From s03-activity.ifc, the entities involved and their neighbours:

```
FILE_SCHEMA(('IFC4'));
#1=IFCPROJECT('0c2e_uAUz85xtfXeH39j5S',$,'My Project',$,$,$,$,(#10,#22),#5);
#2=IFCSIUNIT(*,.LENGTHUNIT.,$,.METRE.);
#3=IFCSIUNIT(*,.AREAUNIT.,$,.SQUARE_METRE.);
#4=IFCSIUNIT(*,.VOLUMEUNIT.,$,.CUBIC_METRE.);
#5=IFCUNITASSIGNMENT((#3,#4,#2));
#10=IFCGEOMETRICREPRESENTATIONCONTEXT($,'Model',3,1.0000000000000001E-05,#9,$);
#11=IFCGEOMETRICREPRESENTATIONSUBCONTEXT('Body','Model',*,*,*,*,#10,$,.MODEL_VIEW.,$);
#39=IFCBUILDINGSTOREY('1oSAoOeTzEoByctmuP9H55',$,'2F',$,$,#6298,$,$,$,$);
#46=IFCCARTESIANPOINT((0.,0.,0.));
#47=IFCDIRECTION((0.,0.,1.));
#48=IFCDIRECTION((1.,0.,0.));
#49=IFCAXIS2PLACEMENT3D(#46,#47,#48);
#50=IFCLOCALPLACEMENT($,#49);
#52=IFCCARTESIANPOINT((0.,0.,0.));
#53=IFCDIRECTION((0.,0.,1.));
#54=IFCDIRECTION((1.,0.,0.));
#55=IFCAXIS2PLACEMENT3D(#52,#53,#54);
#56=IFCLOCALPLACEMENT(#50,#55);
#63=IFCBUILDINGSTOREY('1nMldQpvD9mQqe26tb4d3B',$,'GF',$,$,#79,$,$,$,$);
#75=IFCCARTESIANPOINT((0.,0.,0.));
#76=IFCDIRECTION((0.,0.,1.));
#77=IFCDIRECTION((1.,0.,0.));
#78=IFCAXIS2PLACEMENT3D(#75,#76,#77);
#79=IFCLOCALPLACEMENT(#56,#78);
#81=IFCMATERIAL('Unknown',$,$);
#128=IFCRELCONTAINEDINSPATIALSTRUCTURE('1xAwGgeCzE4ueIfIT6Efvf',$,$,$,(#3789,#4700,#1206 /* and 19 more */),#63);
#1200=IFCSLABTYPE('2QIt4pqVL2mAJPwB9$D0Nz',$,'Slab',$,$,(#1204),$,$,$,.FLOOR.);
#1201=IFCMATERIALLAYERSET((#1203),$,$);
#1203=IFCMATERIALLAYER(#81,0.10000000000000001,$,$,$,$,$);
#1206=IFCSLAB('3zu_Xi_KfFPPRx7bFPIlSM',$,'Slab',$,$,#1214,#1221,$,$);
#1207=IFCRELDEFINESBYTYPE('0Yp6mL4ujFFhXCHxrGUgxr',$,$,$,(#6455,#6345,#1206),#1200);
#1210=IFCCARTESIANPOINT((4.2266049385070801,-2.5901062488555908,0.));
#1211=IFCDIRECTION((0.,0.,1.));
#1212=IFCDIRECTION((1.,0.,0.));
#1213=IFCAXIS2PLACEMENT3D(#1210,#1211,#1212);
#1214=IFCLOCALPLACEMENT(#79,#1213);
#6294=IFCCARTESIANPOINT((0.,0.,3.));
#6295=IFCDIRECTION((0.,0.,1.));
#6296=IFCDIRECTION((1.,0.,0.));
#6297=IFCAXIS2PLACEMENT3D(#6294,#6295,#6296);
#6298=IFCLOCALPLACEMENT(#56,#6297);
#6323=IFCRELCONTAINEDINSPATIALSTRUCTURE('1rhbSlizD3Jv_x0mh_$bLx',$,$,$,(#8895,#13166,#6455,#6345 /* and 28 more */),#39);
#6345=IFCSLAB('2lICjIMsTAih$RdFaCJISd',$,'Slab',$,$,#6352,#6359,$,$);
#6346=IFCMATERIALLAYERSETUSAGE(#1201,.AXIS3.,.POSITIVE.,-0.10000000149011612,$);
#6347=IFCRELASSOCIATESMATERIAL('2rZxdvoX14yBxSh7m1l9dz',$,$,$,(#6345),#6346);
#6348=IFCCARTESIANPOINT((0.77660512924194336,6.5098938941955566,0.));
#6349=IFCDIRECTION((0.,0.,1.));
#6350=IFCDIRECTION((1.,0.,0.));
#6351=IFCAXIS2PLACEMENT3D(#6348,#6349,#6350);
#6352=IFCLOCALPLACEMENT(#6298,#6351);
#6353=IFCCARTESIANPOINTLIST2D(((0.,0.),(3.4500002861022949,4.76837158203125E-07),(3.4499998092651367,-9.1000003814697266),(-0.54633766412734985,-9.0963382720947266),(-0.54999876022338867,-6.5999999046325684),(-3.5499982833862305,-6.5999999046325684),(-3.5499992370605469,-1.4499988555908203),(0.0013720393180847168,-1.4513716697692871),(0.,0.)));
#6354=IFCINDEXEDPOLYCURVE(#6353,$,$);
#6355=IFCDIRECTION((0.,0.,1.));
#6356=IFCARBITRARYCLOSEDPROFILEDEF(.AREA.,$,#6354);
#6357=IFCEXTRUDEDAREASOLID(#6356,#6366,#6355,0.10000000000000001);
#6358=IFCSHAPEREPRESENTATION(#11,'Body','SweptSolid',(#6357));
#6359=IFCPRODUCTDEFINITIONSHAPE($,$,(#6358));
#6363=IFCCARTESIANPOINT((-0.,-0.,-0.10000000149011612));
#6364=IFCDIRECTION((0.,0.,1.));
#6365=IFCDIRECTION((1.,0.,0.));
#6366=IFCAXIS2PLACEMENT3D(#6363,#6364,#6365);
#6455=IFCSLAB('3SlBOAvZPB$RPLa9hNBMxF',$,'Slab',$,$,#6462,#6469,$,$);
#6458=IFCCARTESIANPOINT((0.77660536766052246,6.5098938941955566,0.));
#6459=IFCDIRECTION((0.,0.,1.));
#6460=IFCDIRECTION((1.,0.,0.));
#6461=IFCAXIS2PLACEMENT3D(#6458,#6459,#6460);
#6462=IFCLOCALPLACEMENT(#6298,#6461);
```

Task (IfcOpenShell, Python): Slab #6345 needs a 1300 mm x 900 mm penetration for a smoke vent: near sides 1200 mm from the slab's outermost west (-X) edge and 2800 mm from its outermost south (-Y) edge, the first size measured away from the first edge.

```python
import numpy as np
import ifcopenshell
import ifcopenshell.api.feature
import ifcopenshell.api.geometry
import ifcopenshell.api.root
import ifcopenshell.geom
import ifcopenshell.util.placement
import ifcopenshell.util.representation
import ifcopenshell.util.shape
import ifcopenshell.util.unit

model = ifcopenshell.open("s03-activity.ifc")
unit_scale = ifcopenshell.util.unit.calculate_unit_scale(model)
settings = ifcopenshell.geom.settings()


def volume(element):
    """Net volume in cubic metres, openings subtracted."""
    shape = ifcopenshell.geom.create_shape(settings, element)
    return ifcopenshell.util.shape.get_volume(shape.geometry)


slab = model.by_guid("2lICjIMsTAih$RdFaCJISd")
before = volume(slab)

# Extent in the slab's own axes, in metres. The edges named are its -X and -Y sides.
slab_shape = ifcopenshell.geom.create_shape(settings, slab)
vertices = ifcopenshell.util.shape.get_vertices(slab_shape.geometry)
x_min, y_min, bottom = vertices.min(axis=0)
top = vertices[:, 2].max()

opening = ifcopenshell.api.root.create_entity(model, ifc_class="IfcOpeningElement", name="Smoke vent opening", predefined_type="OPENING")
context = ifcopenshell.util.representation.get_context(model, "Model", "Body", "MODEL_VIEW")
width, depth = 1.3, 0.9
outline = [(0.0, 0.0), (width, 0.0), (width, depth), (0.0, depth), (0.0, 0.0)]
# Overshoot both faces by 50 mm so the cut is clean.
shape = ifcopenshell.api.geometry.add_slab_representation(
    model, context=context, depth=top - bottom + 0.1, polyline=outline
)
ifcopenshell.api.geometry.assign_representation(model, product=opening, representation=shape)

matrix = ifcopenshell.util.placement.get_local_placement(slab.ObjectPlacement)
matrix[:, 3] = matrix @ np.append(np.array([x_min + 1.2, y_min + 2.8, bottom - 0.05]) / unit_scale, 1.0)
ifcopenshell.api.geometry.edit_object_placement(model, product=opening, matrix=matrix, is_si=False)
ifcopenshell.api.feature.add_feature(model, feature=opening, element=slab)

after = volume(slab)

print(f"slab volume {before:.3f} -> {after:.3f} m3")

model.write("s03-activity_rev.ifc")
```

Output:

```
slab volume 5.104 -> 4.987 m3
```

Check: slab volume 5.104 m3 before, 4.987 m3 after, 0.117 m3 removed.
